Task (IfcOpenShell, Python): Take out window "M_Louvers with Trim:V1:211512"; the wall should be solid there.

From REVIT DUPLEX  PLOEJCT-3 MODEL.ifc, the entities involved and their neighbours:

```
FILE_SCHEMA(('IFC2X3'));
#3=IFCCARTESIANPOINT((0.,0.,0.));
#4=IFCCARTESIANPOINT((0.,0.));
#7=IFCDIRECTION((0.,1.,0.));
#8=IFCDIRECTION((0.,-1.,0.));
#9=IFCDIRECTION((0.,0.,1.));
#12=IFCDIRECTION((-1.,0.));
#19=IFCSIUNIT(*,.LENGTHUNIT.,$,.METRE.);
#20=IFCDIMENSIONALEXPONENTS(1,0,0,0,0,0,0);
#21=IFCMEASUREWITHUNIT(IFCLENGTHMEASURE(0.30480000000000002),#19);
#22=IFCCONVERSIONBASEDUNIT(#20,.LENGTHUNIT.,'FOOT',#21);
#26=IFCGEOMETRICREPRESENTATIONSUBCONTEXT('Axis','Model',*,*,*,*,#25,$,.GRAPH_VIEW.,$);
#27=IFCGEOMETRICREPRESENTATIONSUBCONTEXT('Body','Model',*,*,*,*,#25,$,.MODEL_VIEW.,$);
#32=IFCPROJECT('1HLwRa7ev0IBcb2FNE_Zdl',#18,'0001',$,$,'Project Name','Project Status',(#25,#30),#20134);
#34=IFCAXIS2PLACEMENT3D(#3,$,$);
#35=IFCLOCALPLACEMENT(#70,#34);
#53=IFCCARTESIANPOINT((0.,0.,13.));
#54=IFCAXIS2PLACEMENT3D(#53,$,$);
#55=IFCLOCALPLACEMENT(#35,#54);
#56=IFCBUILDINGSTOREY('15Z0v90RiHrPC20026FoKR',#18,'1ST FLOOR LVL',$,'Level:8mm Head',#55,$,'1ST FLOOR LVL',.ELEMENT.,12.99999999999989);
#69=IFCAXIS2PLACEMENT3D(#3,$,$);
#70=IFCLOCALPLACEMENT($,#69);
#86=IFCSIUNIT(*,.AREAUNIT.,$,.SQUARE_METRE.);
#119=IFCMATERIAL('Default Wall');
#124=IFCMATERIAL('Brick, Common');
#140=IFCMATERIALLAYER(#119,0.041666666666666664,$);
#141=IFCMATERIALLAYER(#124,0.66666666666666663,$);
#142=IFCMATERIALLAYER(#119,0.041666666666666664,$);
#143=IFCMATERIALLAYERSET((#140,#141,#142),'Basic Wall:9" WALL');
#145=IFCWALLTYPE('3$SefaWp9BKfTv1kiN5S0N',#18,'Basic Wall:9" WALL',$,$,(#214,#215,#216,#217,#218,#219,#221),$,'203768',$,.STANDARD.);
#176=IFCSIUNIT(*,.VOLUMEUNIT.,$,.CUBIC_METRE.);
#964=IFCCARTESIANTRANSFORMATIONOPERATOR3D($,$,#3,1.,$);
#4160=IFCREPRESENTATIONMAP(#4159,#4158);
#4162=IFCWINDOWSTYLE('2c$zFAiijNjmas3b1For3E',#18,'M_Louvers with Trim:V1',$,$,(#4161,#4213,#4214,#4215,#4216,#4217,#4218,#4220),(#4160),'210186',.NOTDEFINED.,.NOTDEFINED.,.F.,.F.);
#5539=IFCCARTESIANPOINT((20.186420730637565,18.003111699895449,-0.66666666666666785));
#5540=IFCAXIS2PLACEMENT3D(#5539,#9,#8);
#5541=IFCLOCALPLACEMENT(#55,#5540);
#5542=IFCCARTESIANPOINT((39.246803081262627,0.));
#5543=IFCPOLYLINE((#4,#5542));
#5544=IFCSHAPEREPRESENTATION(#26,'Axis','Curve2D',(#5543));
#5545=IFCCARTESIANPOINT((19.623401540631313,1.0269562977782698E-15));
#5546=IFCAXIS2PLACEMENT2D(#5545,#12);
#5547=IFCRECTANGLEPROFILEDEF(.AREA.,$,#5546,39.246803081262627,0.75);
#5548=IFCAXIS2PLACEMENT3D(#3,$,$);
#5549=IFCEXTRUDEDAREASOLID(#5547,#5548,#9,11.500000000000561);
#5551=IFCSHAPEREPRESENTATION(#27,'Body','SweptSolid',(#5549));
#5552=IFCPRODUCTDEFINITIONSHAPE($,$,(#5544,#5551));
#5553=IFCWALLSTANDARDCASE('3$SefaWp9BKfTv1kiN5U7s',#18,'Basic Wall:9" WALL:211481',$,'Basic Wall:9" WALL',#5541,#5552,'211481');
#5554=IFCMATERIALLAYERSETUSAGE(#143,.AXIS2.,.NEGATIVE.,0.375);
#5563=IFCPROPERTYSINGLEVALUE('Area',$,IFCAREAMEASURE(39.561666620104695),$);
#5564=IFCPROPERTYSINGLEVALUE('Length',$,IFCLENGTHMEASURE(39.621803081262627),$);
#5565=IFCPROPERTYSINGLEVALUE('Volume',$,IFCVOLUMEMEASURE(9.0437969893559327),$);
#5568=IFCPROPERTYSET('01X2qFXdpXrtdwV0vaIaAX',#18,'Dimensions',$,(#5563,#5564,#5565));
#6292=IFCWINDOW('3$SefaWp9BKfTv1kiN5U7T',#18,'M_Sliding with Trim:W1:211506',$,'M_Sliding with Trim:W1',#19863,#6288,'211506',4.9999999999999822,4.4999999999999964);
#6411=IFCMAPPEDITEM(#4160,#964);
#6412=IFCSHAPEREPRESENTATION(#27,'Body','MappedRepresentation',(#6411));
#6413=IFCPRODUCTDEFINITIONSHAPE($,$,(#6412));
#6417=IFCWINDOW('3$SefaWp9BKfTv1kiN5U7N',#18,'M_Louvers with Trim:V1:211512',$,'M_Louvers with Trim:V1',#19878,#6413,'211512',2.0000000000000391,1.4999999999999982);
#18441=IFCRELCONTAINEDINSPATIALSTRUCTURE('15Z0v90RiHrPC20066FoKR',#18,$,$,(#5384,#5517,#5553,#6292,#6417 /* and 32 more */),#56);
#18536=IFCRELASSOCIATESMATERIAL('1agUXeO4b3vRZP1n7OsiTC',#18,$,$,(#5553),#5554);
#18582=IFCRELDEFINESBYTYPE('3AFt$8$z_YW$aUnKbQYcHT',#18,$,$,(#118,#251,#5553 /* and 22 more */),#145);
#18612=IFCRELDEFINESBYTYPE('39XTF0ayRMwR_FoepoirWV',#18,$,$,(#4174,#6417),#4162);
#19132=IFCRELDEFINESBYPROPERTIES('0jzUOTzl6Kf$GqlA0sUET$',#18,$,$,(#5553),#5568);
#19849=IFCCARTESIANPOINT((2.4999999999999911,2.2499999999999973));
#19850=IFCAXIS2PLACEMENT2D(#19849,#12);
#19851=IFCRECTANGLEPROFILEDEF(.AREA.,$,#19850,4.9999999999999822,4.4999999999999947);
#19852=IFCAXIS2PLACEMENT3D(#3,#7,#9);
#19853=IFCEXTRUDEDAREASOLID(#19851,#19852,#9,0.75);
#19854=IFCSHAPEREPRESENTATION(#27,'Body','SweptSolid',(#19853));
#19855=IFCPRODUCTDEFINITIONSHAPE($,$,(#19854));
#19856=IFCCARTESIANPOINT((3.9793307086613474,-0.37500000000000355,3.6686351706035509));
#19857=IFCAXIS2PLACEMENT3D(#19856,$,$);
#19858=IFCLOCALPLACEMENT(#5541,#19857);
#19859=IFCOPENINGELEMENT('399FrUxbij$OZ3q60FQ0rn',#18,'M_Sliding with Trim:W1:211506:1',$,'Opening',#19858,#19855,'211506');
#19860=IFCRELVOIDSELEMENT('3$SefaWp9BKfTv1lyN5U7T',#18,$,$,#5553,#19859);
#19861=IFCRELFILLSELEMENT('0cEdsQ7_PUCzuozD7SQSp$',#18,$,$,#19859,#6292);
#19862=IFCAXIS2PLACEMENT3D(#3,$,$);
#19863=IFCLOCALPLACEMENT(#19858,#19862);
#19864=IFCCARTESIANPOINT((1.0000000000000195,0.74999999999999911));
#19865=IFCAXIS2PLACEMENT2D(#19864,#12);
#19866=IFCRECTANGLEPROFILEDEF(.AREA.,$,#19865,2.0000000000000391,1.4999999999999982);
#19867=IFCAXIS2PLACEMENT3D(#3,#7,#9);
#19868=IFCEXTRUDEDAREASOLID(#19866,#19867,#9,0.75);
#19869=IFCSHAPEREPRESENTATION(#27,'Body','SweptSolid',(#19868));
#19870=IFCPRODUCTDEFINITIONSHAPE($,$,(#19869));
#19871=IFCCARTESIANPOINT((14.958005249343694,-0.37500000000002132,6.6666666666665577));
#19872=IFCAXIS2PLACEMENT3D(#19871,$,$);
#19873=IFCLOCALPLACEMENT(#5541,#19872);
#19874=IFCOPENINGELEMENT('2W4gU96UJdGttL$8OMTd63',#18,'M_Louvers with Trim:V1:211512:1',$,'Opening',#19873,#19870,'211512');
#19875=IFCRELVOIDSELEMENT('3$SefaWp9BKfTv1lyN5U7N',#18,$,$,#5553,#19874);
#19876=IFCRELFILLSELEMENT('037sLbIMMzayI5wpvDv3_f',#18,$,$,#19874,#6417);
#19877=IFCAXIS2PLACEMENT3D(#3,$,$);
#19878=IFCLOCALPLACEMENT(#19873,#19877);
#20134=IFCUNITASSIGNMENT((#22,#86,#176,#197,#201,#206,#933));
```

```python
import ifcopenshell
import ifcopenshell.api.feature
import ifcopenshell.api.pset
import ifcopenshell.api.root
import ifcopenshell.geom
import ifcopenshell.util.element
import ifcopenshell.util.shape
import ifcopenshell.util.unit

model = ifcopenshell.open("REVIT DUPLEX  PLOEJCT-3 MODEL.ifc")
area_scale = ifcopenshell.util.unit.calculate_unit_scale(model, "AREAUNIT")
volume_scale = ifcopenshell.util.unit.calculate_unit_scale(model, "VOLUMEUNIT")
settings = ifcopenshell.geom.settings()


def volume(element):
    """Net volume in cubic metres, openings subtracted."""
    shape = ifcopenshell.geom.create_shape(settings, element)
    return ifcopenshell.util.shape.get_volume(shape.geometry)


window = model.by_guid("3$SefaWp9BKfTv1kiN5U7N")
opening = window.FillsVoids[0].RelatingOpeningElement
wall = opening.VoidsElements[0].RelatingBuildingElement
before = volume(wall)

ifcopenshell.api.root.remove_product(model, product=window)
ifcopenshell.api.feature.remove_feature(model, feature=opening)

after = volume(wall)
thickness = 0.2286  # wall thickness in metres

# Update the wall's stored quantities.
pset = model.by_id(ifcopenshell.util.element.get_pset(wall, "Dimensions", should_inherit=False)["id"])
ifcopenshell.api.pset.edit_pset(model, pset=pset, properties={
    "Area": model.create_entity("IfcAreaMeasure", after / thickness / area_scale),
    "Volume": model.create_entity("IfcVolumeMeasure", after / volume_scale),
})

print(f"wall volume {before:.3f} -> {after:.3f} m3")

model.write("REVIT DUPLEX  PLOEJCT-3 MODEL_v2.ifc")
```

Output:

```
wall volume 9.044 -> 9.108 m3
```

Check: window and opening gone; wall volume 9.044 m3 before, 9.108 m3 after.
